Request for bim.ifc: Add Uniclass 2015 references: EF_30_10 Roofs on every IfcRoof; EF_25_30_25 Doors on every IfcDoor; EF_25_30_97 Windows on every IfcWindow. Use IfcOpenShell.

First a look at what the model holds.

```python
import ifcopenshell

model = ifcopenshell.open("bim.ifc")
print(model.schema)
print("classifications:", [c.Name for c in model.by_type("IfcClassification")])
for ifc_class in ("IfcDoor", "IfcRoof", "IfcStair", "IfcWall", "IfcWindow"):
    print(ifc_class, len(model.by_type(ifc_class)))
```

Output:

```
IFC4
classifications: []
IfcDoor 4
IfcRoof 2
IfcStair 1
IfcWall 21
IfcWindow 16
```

```python
import ifcopenshell
import ifcopenshell.api.classification

model = ifcopenshell.open("bim.ifc")

system = ifcopenshell.api.classification.add_classification(model, classification="Uniclass 2015")

codes = {
    "IfcRoof": ("EF_30_10", "Roofs"),
    "IfcDoor": ("EF_25_30_25", "Doors"),
    "IfcWindow": ("EF_25_30_97", "Windows"),
}
for ifc_class, (code, name) in codes.items():
    products = model.by_type(ifc_class)
    ifcopenshell.api.classification.add_reference(
        model, products=products, classification=system, identification=code, name=name
    )
    print(code, len(products))

model.write("bim_rev.ifc")
```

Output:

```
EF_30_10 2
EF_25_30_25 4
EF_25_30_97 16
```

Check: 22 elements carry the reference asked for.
